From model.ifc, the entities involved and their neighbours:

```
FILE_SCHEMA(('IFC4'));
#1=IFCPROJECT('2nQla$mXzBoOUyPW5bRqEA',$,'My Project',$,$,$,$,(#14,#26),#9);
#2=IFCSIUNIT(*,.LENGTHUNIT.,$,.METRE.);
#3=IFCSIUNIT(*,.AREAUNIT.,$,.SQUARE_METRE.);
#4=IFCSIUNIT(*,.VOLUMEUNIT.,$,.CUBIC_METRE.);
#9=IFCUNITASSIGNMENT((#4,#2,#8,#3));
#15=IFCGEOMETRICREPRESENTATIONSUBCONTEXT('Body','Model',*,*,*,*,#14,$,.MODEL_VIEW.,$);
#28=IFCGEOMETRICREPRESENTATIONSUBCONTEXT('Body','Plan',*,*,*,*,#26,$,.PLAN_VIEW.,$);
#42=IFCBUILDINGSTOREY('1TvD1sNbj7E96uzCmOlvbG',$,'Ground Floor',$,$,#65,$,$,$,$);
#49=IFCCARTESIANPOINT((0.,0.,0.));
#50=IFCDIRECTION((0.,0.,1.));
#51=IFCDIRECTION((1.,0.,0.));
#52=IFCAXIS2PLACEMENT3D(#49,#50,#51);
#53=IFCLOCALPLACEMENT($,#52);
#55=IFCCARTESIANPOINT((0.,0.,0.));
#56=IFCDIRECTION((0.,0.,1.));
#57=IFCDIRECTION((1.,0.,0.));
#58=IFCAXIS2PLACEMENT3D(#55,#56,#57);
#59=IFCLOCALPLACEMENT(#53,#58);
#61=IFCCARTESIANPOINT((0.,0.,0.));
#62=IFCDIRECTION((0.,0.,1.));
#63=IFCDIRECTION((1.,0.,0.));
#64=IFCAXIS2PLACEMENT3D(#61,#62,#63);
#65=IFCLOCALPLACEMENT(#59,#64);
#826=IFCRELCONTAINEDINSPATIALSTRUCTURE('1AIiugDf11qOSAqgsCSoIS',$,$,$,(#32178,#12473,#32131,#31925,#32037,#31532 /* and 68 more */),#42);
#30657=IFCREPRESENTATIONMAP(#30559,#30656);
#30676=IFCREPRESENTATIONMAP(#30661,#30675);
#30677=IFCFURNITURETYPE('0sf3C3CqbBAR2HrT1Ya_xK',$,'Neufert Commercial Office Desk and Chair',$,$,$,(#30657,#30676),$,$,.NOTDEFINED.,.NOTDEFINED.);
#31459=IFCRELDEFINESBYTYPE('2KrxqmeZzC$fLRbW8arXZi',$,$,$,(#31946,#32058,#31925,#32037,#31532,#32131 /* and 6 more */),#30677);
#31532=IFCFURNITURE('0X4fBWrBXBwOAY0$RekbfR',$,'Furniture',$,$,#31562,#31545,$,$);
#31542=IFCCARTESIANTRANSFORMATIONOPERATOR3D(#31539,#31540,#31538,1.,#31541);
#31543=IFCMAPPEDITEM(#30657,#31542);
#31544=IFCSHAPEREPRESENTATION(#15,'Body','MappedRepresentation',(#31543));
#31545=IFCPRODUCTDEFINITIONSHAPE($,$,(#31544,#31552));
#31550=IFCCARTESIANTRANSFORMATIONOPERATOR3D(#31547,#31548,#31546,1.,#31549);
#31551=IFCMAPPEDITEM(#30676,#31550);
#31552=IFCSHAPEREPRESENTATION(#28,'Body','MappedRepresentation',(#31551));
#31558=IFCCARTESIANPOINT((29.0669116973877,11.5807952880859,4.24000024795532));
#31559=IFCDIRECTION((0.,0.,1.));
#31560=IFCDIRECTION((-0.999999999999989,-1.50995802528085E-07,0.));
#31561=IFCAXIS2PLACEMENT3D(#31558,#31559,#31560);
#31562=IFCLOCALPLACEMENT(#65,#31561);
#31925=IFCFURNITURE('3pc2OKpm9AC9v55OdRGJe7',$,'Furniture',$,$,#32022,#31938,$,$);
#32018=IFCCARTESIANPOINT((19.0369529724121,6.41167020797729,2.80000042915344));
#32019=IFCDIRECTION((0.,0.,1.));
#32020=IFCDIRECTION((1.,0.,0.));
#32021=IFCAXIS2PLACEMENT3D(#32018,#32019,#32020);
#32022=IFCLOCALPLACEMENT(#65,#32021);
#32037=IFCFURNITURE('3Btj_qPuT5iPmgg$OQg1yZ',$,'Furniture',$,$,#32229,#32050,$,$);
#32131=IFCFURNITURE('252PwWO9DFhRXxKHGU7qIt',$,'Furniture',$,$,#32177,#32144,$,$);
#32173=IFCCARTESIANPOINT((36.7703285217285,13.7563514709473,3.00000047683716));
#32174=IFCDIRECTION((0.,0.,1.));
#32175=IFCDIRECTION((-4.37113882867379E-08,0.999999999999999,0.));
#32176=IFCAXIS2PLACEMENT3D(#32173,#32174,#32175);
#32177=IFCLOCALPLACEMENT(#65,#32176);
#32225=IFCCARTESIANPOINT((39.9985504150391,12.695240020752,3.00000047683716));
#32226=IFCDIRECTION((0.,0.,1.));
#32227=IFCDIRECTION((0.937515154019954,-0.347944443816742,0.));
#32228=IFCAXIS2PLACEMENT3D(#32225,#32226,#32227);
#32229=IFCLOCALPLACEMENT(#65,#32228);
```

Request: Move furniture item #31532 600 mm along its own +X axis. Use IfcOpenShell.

```python
import ifcopenshell
import ifcopenshell.api.geometry
import ifcopenshell.util.placement

model = ifcopenshell.open("model.ifc")

item = model.by_guid("0X4fBWrBXBwOAY0$RekbfR")
matrix = ifcopenshell.util.placement.get_local_placement(item.ObjectPlacement)
matrix[:3, 3] += matrix[:3, 0] * 0.6
ifcopenshell.api.geometry.edit_object_placement(model, product=item, matrix=matrix, is_si=False)

print(ifcopenshell.util.placement.get_local_placement(item.ObjectPlacement).round(3) + 0.0)

model.write("model_edited.ifc")
```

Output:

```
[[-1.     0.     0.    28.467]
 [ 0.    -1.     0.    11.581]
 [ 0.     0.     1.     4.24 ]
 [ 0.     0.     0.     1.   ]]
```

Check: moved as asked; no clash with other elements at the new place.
